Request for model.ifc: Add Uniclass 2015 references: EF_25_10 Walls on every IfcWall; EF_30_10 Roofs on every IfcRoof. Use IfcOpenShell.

First a look at what the model holds.

```python
import ifcopenshell

model = ifcopenshell.open("model.ifc")
print(model.schema)
print("classifications:", [c.Name for c in model.by_type("IfcClassification")])
for ifc_class in ("IfcDoor", "IfcRoof", "IfcStair", "IfcWall", "IfcWindow"):
    print(ifc_class, len(model.by_type(ifc_class)))
```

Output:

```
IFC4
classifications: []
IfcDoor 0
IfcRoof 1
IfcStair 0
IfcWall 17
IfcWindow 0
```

```python
import ifcopenshell
import ifcopenshell.api.classification

model = ifcopenshell.open("model.ifc")

system = ifcopenshell.api.classification.add_classification(model, classification="Uniclass 2015")

codes = {
    "IfcWall": ("EF_25_10", "Walls"),
    "IfcRoof": ("EF_30_10", "Roofs"),
}
for ifc_class, (code, name) in codes.items():
    products = model.by_type(ifc_class)
    ifcopenshell.api.classification.add_reference(
        model, products=products, classification=system, identification=code, name=name
    )
    print(code, len(products))

model.write("model_v2.ifc")
```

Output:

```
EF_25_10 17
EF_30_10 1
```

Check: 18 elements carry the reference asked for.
